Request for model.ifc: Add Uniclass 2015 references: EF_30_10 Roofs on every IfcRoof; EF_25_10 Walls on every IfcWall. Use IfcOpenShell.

First a look at what the model holds.

```python
import ifcopenshell

model = ifcopenshell.open("model.ifc")
print(model.schema)
print("classifications:", [c.Name for c in model.by_type("IfcClassification")])
for ifc_class in ("IfcDoor", "IfcRoof", "IfcStair", "IfcWall", "IfcWindow"):
    print(ifc_class, len(model.by_type(ifc_class)))
```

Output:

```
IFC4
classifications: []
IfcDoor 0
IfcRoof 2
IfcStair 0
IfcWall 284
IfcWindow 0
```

```python
import ifcopenshell
import ifcopenshell.api.classification

model = ifcopenshell.open("model.ifc")

system = ifcopenshell.api.classification.add_classification(model, classification="Uniclass 2015")

codes = {
    "IfcRoof": ("EF_30_10", "Roofs"),
    "IfcWall": ("EF_25_10", "Walls"),
}
for ifc_class, (code, name) in codes.items():
    products = model.by_type(ifc_class)
    ifcopenshell.api.classification.add_reference(
        model, products=products, classification=system, identification=code, name=name
    )
    print(code, len(products))

model.write("model_updated.ifc")
```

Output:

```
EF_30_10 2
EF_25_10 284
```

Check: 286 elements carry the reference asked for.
